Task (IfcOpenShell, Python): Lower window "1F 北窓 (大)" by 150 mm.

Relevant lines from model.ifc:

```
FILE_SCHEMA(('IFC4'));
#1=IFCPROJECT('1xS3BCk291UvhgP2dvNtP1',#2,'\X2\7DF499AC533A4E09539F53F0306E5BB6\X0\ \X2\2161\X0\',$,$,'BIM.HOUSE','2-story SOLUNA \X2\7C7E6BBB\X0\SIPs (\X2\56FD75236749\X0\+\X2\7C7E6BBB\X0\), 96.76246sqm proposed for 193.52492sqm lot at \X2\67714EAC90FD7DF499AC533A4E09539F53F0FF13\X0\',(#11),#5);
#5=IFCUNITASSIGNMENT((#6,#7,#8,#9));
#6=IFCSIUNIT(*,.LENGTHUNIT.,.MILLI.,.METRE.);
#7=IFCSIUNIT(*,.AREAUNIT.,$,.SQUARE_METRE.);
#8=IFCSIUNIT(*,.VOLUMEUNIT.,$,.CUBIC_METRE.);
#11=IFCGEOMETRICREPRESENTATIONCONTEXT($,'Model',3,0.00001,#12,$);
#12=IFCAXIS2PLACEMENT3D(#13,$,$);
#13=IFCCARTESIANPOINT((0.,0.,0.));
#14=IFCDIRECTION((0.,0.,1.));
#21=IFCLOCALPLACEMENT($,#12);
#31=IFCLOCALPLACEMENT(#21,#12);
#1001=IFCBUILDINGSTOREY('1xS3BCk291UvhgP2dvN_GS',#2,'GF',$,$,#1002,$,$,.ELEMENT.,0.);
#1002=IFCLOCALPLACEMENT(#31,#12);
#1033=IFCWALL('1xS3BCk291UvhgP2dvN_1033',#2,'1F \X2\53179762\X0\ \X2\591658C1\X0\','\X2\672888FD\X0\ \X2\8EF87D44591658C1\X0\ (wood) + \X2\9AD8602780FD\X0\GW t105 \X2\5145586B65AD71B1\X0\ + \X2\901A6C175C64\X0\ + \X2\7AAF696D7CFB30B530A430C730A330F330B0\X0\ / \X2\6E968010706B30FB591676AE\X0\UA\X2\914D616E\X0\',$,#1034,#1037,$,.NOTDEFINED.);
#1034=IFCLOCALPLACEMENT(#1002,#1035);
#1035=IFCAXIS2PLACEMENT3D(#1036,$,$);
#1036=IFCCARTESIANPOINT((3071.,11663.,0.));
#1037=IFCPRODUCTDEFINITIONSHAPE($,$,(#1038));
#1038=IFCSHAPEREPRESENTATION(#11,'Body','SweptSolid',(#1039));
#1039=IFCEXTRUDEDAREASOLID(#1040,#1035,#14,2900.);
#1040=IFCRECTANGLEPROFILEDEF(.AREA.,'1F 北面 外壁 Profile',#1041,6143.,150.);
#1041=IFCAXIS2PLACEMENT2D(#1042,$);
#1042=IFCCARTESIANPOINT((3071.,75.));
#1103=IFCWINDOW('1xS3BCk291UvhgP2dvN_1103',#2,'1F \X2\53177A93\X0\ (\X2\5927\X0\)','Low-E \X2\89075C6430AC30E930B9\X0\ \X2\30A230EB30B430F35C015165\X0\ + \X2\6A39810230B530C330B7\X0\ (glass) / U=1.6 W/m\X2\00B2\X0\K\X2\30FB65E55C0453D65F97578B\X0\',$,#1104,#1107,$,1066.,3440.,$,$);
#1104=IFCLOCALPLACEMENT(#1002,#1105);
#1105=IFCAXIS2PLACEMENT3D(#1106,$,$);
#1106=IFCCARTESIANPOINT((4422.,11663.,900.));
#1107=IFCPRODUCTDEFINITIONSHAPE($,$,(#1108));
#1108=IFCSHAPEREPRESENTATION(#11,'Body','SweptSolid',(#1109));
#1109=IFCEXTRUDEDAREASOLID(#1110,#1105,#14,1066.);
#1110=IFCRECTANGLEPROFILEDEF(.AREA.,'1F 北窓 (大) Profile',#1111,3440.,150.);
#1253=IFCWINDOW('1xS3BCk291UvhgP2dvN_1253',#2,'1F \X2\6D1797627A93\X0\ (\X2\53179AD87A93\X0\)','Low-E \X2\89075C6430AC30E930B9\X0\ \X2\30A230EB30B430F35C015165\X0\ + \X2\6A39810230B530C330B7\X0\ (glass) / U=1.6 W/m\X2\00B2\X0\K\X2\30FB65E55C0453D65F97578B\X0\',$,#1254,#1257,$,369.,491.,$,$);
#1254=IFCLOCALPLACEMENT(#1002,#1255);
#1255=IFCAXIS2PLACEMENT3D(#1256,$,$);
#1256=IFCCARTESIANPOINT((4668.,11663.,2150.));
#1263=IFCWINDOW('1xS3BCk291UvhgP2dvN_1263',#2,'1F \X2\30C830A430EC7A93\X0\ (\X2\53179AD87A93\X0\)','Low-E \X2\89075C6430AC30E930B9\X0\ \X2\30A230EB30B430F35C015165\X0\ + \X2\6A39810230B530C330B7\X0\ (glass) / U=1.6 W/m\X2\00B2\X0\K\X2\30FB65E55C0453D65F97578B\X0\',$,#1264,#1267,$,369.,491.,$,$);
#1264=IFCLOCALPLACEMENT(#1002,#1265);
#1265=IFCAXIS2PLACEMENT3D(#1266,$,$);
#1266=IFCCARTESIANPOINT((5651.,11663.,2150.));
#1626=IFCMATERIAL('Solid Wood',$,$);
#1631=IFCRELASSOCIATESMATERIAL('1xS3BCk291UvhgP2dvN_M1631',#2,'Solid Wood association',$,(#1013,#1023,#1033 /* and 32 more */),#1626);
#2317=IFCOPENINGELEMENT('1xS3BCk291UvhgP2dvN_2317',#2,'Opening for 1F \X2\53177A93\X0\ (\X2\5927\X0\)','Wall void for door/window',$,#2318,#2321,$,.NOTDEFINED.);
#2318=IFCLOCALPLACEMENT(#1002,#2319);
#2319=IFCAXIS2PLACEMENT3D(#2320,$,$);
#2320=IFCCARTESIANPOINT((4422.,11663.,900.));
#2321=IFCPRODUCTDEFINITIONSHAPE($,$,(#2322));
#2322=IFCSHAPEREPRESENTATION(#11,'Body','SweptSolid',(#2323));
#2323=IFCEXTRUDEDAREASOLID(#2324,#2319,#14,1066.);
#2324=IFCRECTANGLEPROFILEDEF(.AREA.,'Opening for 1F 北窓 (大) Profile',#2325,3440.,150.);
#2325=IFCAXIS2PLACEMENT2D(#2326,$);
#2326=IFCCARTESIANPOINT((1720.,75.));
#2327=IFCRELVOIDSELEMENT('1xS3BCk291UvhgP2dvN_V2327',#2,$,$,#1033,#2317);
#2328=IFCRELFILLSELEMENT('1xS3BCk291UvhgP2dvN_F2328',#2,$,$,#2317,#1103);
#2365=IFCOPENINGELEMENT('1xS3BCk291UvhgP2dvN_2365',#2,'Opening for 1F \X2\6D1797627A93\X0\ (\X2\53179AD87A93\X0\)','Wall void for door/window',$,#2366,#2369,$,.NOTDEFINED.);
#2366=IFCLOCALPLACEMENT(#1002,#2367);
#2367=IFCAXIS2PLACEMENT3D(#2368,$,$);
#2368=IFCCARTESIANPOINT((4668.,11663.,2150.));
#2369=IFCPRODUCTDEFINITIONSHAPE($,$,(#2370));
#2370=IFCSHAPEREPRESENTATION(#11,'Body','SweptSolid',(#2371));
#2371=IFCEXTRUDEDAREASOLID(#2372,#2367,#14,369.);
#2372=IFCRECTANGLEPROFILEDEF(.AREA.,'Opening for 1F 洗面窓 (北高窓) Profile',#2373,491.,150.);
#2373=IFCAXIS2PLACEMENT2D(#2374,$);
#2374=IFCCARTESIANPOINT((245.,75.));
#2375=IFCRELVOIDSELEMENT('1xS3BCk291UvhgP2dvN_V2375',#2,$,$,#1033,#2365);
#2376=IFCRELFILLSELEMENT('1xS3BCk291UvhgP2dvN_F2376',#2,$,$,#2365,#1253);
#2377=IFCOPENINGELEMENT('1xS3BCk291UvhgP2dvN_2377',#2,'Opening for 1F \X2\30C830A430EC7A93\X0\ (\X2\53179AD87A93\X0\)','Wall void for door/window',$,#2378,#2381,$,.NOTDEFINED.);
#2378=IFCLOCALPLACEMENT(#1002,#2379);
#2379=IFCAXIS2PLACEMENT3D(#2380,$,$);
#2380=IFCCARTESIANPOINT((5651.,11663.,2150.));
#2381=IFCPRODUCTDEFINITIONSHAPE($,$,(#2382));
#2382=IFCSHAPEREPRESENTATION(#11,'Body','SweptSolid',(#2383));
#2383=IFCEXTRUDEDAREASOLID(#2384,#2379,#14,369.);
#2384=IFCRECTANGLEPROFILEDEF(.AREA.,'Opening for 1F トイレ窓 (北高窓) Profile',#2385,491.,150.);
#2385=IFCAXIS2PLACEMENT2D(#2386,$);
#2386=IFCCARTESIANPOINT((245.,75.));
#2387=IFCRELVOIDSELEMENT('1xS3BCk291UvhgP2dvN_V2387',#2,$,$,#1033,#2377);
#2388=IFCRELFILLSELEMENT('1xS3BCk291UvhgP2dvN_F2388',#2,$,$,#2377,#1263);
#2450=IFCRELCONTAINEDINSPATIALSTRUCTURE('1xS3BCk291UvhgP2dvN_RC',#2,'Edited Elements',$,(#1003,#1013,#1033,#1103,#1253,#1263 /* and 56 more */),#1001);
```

```python
import numpy as np
import ifcopenshell
import ifcopenshell.api.geometry
import ifcopenshell.util.placement
import ifcopenshell.util.unit

model = ifcopenshell.open("model.ifc")
unit_scale = ifcopenshell.util.unit.calculate_unit_scale(model)

window = model.by_guid("1xS3BCk291UvhgP2dvN_1103")
opening = window.FillsVoids[0].RelatingOpeningElement
dz = -0.15 / unit_scale

shift = np.array([0.0, 0.0, dz])
# The window is not placed relative to its opening, so move both.
for product in (opening, window):
    matrix = ifcopenshell.util.placement.get_local_placement(product.ObjectPlacement)
    matrix[:3, 3] += shift
    ifcopenshell.api.geometry.edit_object_placement(model, product=product, matrix=matrix, is_si=False)

print(f"moved by {dz * unit_scale:+.3f} m")

model.write("model_rev.ifc")
```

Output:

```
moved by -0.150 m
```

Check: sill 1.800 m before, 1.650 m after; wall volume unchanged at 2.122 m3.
